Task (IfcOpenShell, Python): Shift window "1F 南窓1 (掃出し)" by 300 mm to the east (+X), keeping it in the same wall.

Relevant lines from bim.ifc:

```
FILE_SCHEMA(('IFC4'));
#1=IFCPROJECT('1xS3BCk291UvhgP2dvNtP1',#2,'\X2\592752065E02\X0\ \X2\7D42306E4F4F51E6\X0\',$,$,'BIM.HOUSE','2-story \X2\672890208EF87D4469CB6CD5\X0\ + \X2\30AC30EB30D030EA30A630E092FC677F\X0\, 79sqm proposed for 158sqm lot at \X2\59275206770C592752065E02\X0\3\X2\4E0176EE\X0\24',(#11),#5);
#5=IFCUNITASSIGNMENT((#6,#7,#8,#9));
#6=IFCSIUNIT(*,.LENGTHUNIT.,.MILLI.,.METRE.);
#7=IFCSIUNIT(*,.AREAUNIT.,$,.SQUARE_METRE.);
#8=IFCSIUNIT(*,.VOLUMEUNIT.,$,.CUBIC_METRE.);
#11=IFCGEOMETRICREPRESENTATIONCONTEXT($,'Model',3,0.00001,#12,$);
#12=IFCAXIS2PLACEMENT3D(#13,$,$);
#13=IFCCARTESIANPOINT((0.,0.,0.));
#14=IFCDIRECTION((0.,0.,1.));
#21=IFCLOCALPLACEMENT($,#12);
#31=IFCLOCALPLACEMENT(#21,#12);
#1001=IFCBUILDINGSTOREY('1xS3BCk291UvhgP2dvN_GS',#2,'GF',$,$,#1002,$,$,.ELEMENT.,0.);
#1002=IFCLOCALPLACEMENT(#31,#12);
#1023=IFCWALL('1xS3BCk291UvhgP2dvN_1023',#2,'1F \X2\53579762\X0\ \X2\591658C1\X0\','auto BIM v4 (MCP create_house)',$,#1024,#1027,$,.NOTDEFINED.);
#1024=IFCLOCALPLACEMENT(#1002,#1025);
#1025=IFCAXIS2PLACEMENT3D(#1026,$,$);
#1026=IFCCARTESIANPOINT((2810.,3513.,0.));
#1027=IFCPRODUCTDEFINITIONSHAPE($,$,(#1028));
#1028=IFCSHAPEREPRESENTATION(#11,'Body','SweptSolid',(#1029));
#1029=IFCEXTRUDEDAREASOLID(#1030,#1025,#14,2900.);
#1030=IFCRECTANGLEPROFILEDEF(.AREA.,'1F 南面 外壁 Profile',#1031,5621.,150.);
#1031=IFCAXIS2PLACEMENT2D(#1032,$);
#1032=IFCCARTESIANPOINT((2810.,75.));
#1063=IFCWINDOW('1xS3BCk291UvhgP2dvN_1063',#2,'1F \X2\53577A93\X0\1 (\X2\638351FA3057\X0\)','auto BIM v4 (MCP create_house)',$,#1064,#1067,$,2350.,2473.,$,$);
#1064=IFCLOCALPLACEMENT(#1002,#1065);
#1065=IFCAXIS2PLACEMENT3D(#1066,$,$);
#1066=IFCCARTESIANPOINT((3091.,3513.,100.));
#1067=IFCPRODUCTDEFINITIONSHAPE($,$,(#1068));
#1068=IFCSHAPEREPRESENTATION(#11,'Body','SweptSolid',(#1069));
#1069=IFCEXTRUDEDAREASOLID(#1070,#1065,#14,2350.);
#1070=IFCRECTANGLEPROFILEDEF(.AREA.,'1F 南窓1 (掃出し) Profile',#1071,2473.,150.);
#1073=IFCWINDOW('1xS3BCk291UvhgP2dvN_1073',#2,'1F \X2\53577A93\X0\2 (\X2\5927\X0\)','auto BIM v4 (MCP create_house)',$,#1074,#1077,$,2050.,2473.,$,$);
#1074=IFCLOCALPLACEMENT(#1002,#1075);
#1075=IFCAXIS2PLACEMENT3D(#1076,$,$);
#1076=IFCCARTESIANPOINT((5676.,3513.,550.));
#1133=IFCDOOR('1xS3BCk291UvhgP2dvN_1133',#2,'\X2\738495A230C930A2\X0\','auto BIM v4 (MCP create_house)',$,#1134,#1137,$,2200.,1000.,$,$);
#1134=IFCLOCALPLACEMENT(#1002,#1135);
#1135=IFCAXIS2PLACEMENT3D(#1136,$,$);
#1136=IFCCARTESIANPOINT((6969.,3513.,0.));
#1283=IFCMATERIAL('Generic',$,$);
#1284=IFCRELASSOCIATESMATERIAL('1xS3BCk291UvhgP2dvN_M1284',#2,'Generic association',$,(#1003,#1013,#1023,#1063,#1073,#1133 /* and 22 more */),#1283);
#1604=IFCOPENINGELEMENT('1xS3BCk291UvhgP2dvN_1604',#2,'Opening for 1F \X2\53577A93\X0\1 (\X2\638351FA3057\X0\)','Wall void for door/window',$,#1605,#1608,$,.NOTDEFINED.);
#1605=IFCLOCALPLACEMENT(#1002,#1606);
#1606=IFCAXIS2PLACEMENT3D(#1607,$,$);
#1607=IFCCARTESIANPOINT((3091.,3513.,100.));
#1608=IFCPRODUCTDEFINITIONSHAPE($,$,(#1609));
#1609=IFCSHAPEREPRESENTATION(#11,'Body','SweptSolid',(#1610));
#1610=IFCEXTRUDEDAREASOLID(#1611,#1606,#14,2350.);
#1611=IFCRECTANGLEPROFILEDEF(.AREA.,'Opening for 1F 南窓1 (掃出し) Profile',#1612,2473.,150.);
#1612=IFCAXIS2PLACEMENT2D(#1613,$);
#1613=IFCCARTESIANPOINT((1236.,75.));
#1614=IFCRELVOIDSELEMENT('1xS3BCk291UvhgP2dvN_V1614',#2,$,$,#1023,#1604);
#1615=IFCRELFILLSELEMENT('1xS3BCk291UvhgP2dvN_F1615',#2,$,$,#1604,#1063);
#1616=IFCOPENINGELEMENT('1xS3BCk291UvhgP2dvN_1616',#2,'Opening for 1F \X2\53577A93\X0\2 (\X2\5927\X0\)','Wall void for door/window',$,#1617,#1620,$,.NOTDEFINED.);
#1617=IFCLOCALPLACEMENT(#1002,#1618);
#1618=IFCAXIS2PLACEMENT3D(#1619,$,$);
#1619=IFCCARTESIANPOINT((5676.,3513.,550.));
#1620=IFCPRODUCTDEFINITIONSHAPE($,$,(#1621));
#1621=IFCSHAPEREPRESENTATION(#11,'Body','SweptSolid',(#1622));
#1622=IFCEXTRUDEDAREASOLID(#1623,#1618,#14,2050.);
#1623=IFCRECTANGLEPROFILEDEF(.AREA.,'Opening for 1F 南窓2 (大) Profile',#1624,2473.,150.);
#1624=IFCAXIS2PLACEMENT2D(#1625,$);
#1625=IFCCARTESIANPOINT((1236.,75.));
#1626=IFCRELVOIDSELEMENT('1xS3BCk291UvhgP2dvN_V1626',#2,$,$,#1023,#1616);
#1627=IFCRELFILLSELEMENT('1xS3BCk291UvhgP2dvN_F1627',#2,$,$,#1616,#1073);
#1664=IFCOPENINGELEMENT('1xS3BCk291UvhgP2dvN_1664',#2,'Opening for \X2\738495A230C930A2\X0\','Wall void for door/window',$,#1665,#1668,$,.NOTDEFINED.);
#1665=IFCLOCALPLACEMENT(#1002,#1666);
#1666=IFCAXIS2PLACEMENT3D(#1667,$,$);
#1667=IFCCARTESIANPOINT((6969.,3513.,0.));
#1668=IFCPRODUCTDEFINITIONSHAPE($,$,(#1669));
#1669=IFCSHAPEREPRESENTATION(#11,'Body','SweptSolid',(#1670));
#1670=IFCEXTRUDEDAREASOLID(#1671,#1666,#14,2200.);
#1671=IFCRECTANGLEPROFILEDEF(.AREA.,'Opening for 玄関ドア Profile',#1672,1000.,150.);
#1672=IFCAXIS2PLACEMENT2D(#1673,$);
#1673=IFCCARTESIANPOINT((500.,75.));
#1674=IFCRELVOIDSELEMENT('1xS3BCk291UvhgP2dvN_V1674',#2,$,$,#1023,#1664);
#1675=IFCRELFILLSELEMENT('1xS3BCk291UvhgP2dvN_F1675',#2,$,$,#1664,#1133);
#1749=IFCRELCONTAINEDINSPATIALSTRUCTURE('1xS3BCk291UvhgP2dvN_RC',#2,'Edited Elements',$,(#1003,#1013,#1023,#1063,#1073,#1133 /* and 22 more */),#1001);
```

```python
import ifcopenshell
import ifcopenshell.api.geometry
import ifcopenshell.util.placement

model = ifcopenshell.open("bim.ifc")

window = model.by_guid("1xS3BCk291UvhgP2dvN_1063")
opening = window.FillsVoids[0].RelatingOpeningElement
wall = opening.VoidsElements[0].RelatingBuildingElement

wall_matrix = ifcopenshell.util.placement.get_local_placement(wall.ObjectPlacement)
shift = wall_matrix[:3, 0] * 300.0
before = ifcopenshell.util.placement.get_local_placement(window.ObjectPlacement)[:3, 3].copy()

# The window is not placed relative to its opening, so move both.
for product in (opening, window):
    matrix = ifcopenshell.util.placement.get_local_placement(product.ObjectPlacement)
    matrix[:3, 3] += shift
    ifcopenshell.api.geometry.edit_object_placement(model, product=product, matrix=matrix, is_si=False)

after = ifcopenshell.util.placement.get_local_placement(window.ObjectPlacement)[:3, 3]
print("window moved by", (after - before).round(3) + 0.0)

model.write("bim_updated.ifc")
```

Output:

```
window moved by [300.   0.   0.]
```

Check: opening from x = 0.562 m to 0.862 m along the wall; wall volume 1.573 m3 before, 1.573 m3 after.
